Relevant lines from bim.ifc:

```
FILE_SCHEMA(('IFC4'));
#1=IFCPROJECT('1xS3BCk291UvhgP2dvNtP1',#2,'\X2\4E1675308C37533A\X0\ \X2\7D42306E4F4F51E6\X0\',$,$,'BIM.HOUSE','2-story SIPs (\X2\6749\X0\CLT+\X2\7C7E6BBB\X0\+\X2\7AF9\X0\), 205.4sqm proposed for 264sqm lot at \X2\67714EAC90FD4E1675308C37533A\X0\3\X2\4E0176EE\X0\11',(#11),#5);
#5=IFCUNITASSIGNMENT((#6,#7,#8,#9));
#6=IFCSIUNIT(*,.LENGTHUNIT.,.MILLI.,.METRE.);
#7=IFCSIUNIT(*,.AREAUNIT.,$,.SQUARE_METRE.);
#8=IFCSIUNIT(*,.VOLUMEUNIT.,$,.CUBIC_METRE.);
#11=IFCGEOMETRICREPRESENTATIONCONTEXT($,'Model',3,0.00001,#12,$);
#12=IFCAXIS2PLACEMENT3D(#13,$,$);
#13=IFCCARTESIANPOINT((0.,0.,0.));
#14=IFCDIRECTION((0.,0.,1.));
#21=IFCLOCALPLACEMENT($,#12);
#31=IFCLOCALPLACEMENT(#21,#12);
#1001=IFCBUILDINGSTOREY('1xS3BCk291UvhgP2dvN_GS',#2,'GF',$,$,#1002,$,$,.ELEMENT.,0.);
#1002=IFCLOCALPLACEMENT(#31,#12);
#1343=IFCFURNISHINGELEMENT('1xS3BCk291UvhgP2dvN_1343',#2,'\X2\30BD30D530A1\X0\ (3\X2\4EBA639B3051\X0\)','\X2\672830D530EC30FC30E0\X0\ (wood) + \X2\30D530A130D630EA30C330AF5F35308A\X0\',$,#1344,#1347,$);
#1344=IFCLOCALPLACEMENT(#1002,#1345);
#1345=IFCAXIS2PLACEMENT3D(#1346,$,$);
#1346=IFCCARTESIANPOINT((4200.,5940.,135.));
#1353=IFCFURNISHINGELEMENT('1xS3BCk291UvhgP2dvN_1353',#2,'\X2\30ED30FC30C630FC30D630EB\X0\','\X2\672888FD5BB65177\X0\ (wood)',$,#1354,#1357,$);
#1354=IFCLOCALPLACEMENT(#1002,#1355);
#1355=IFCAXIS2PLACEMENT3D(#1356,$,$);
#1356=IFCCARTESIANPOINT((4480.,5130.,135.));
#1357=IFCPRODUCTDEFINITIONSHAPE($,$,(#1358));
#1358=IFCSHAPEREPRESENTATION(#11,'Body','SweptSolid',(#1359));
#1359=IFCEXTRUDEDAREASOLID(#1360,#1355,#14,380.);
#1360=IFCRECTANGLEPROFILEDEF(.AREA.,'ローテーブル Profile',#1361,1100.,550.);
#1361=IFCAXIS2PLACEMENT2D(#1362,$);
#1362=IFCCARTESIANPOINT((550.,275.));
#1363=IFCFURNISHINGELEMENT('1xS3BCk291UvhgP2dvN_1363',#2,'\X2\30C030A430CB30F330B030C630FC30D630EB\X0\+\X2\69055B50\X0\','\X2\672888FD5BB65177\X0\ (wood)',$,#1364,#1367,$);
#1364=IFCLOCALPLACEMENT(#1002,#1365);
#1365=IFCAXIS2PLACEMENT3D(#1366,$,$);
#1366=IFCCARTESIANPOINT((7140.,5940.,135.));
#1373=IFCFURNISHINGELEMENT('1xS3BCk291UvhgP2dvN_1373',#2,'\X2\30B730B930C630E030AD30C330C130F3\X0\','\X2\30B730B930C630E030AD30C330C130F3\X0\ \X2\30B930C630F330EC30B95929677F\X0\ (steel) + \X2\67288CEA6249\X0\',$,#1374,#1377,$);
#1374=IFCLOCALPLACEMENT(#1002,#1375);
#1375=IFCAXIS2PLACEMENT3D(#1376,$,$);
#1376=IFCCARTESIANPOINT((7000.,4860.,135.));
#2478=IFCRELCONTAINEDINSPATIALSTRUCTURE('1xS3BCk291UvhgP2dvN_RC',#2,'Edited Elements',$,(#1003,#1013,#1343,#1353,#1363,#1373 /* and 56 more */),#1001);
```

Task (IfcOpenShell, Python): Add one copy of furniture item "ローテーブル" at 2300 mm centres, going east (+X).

```python
import numpy as np
import ifcopenshell
import ifcopenshell.api.geometry
import ifcopenshell.api.root
import ifcopenshell.util.element
import ifcopenshell.util.placement

model = ifcopenshell.open("bim.ifc")


def reuse_history(source, copy):
    """copy_class also copies each property set's owner history, people and application; keep the originals."""
    for rel in copy.IsDefinedBy:
        if rel.is_a("IfcRelDefinesByProperties") and (history := rel.RelatingPropertyDefinition.OwnerHistory):
            rel.RelatingPropertyDefinition.OwnerHistory = source.OwnerHistory
            ifcopenshell.util.element.remove_deep2(model, history)


source = model.by_guid("1xS3BCk291UvhgP2dvN_1353")
base = ifcopenshell.util.placement.get_local_placement(source.ObjectPlacement)
step = np.array([1.0, 0.0, 0.0]) * 2300.0

for i in range(1, 2):
    copy = ifcopenshell.api.root.copy_class(model, product=source)
    copy.Representation = ifcopenshell.util.element.copy_deep(
        model, source.Representation, exclude=["IfcGeometricRepresentationContext", "IfcRepresentationMap"]
    )
    reuse_history(source, copy)
    matrix = base.copy()
    matrix[:3, 3] += i * step
    print("added at", matrix[:3, 3].round(3) + 0.0)
    ifcopenshell.api.geometry.edit_object_placement(model, product=copy, matrix=matrix, is_si=False)

model.write("bim_updated.ifc")
```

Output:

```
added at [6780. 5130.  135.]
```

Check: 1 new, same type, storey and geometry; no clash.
